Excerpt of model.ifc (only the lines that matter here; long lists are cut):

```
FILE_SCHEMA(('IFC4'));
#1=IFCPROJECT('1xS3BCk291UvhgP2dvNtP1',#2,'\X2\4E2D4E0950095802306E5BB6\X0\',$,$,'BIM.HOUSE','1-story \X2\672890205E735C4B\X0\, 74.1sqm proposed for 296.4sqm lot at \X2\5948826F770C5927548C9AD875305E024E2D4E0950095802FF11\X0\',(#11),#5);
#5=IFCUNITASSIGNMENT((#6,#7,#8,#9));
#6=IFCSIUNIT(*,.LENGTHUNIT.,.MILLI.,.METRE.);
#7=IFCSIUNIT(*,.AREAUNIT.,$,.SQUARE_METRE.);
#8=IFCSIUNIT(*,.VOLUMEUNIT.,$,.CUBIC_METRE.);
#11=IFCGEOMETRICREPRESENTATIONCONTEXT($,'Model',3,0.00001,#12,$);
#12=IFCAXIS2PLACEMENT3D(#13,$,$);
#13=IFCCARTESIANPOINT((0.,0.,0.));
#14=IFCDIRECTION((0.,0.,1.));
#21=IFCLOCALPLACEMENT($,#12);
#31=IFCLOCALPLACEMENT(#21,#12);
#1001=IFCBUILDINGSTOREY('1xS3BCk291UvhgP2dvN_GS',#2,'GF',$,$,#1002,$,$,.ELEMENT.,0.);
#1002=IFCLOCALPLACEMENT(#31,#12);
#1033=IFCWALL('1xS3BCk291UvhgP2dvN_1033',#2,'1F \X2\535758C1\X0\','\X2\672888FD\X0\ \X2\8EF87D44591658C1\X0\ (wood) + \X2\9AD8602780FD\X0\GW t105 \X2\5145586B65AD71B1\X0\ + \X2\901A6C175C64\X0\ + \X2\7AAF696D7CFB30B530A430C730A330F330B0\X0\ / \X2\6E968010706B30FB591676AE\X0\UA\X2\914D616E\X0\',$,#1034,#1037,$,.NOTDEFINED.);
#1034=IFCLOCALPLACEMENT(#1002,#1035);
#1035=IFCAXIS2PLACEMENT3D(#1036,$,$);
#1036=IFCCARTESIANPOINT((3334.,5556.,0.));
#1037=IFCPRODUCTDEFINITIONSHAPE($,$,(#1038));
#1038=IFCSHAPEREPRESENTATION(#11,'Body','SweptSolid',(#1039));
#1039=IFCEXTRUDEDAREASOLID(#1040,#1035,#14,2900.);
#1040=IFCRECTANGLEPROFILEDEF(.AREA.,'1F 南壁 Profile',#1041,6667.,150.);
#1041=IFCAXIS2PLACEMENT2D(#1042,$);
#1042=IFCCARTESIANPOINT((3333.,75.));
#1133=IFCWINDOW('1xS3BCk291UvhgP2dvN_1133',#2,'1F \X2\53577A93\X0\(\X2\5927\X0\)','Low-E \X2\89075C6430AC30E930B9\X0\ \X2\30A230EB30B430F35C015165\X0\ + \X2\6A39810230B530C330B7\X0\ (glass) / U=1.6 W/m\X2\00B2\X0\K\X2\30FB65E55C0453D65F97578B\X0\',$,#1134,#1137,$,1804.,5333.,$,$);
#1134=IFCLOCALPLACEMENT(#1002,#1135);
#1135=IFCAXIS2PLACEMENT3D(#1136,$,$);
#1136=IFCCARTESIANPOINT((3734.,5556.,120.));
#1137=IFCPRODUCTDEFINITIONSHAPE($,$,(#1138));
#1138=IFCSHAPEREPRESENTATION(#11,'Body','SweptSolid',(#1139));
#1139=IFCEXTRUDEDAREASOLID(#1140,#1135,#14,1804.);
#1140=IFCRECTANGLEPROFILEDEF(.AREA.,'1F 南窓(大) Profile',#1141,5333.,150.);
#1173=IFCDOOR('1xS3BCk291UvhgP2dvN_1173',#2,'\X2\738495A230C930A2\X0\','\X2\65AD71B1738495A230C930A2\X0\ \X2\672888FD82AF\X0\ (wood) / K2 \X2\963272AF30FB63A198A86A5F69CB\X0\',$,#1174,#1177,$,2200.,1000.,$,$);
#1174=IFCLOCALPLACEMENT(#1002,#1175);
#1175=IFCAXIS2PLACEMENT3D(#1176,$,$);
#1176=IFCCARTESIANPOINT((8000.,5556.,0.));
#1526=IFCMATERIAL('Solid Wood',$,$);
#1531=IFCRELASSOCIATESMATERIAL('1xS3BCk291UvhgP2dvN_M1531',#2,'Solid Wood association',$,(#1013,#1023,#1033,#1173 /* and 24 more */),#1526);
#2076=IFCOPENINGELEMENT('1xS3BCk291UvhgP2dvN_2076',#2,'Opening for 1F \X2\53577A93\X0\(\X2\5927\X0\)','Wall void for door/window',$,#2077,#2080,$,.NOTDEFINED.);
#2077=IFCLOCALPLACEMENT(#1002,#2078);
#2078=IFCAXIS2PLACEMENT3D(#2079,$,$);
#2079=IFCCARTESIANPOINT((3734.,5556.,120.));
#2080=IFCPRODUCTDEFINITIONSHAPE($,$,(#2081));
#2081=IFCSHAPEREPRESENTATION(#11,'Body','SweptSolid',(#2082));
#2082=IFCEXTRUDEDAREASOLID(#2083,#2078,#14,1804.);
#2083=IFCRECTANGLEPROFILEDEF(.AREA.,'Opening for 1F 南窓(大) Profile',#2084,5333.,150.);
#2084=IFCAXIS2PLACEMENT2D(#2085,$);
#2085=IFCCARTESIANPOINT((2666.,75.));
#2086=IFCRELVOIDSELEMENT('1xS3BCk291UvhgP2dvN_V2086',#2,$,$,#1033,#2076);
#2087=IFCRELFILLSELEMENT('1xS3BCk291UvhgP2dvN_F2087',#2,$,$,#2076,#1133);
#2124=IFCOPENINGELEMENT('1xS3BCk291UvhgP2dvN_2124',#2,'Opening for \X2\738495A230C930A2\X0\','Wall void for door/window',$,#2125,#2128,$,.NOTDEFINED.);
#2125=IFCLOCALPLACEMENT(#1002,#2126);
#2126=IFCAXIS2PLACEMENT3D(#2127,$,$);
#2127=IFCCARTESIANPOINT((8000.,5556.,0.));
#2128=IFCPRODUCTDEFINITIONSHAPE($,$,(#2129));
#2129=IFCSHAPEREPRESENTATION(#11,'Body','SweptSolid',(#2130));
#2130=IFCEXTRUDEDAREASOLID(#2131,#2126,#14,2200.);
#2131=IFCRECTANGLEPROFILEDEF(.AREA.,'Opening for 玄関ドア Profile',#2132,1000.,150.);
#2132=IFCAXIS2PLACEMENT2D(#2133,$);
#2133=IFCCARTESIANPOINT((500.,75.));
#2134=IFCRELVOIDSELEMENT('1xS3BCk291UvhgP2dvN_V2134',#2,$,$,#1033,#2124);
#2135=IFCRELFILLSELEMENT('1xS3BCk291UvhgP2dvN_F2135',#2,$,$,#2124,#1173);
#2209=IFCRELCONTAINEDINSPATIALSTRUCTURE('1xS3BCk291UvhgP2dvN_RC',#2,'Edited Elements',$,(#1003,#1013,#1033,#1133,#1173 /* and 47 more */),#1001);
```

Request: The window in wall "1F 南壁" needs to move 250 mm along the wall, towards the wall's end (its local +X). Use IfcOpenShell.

```python
import ifcopenshell
import ifcopenshell.api.geometry
import ifcopenshell.util.placement
import ifcopenshell.util.unit

model = ifcopenshell.open("model.ifc")
unit_scale = ifcopenshell.util.unit.calculate_unit_scale(model)

window = model.by_guid("1xS3BCk291UvhgP2dvN_1133")
opening = window.FillsVoids[0].RelatingOpeningElement
wall = opening.VoidsElements[0].RelatingBuildingElement

wall_matrix = ifcopenshell.util.placement.get_local_placement(wall.ObjectPlacement)
shift = wall_matrix[:3, 0] * 0.25 / unit_scale
before = ifcopenshell.util.placement.get_local_placement(window.ObjectPlacement)[:3, 3].copy()

# The window is not placed relative to its opening, so move both.
for product in (opening, window):
    matrix = ifcopenshell.util.placement.get_local_placement(product.ObjectPlacement)
    matrix[:3, 3] += shift
    ifcopenshell.api.geometry.edit_object_placement(model, product=product, matrix=matrix, is_si=False)

after = ifcopenshell.util.placement.get_local_placement(window.ObjectPlacement)[:3, 3]
print("window moved by", (after - before).round(3) + 0.0)

model.write("model_rev.ifc")
```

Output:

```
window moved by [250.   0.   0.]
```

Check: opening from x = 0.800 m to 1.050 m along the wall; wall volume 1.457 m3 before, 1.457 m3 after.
